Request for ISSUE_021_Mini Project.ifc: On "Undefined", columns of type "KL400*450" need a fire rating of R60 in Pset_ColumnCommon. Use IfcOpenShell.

First a look at what the model holds.

```python
import ifcopenshell
import ifcopenshell.util.element

model = ifcopenshell.open("ISSUE_021_Mini Project.ifc")
print(model.schema)
storey = next(s for s in model.by_type("IfcBuildingStorey") if s.Name == "Undefined")
columns = [e for e in ifcopenshell.util.element.get_decomposition(storey) if e.is_a("IfcColumn")]
seen = {}
for e in columns:
    element_type = ifcopenshell.util.element.get_type(e)
    key = (element_type.Name if element_type != e and element_type else None, ifcopenshell.util.element.get_pset(e, "Pset_ColumnCommon", "FireRating"))
    seen[key] = seen.get(key, 0) + 1
for (name, value), count in sorted(seen.items(), key=str):
    print(count, "x", name, "|", value)
```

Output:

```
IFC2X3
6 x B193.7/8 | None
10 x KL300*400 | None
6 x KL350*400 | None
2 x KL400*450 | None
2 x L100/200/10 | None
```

```python
import ifcopenshell
import ifcopenshell.api.pset
import ifcopenshell.util.element

model = ifcopenshell.open("ISSUE_021_Mini Project.ifc")

storey = next(s for s in model.by_type("IfcBuildingStorey") if s.Name == "Undefined")
columns = [e for e in ifcopenshell.util.element.get_decomposition(storey) if e.is_a("IfcColumn")]

count = 0
for e in columns:
    element_type = ifcopenshell.util.element.get_type(e)
    if element_type in (None, e) or element_type.Name != "KL400*450":
        continue
    # add_pset returns the element's existing set when there is one.
    pset = ifcopenshell.api.pset.add_pset(model, product=e, name="Pset_ColumnCommon")
    ifcopenshell.api.pset.edit_pset(model, pset=pset, properties={"FireRating": "R60"})
    count += 1

print(count, "columns updated")

model.write("ISSUE_021_Mini Project_rev.ifc")
```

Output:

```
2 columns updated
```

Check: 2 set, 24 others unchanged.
